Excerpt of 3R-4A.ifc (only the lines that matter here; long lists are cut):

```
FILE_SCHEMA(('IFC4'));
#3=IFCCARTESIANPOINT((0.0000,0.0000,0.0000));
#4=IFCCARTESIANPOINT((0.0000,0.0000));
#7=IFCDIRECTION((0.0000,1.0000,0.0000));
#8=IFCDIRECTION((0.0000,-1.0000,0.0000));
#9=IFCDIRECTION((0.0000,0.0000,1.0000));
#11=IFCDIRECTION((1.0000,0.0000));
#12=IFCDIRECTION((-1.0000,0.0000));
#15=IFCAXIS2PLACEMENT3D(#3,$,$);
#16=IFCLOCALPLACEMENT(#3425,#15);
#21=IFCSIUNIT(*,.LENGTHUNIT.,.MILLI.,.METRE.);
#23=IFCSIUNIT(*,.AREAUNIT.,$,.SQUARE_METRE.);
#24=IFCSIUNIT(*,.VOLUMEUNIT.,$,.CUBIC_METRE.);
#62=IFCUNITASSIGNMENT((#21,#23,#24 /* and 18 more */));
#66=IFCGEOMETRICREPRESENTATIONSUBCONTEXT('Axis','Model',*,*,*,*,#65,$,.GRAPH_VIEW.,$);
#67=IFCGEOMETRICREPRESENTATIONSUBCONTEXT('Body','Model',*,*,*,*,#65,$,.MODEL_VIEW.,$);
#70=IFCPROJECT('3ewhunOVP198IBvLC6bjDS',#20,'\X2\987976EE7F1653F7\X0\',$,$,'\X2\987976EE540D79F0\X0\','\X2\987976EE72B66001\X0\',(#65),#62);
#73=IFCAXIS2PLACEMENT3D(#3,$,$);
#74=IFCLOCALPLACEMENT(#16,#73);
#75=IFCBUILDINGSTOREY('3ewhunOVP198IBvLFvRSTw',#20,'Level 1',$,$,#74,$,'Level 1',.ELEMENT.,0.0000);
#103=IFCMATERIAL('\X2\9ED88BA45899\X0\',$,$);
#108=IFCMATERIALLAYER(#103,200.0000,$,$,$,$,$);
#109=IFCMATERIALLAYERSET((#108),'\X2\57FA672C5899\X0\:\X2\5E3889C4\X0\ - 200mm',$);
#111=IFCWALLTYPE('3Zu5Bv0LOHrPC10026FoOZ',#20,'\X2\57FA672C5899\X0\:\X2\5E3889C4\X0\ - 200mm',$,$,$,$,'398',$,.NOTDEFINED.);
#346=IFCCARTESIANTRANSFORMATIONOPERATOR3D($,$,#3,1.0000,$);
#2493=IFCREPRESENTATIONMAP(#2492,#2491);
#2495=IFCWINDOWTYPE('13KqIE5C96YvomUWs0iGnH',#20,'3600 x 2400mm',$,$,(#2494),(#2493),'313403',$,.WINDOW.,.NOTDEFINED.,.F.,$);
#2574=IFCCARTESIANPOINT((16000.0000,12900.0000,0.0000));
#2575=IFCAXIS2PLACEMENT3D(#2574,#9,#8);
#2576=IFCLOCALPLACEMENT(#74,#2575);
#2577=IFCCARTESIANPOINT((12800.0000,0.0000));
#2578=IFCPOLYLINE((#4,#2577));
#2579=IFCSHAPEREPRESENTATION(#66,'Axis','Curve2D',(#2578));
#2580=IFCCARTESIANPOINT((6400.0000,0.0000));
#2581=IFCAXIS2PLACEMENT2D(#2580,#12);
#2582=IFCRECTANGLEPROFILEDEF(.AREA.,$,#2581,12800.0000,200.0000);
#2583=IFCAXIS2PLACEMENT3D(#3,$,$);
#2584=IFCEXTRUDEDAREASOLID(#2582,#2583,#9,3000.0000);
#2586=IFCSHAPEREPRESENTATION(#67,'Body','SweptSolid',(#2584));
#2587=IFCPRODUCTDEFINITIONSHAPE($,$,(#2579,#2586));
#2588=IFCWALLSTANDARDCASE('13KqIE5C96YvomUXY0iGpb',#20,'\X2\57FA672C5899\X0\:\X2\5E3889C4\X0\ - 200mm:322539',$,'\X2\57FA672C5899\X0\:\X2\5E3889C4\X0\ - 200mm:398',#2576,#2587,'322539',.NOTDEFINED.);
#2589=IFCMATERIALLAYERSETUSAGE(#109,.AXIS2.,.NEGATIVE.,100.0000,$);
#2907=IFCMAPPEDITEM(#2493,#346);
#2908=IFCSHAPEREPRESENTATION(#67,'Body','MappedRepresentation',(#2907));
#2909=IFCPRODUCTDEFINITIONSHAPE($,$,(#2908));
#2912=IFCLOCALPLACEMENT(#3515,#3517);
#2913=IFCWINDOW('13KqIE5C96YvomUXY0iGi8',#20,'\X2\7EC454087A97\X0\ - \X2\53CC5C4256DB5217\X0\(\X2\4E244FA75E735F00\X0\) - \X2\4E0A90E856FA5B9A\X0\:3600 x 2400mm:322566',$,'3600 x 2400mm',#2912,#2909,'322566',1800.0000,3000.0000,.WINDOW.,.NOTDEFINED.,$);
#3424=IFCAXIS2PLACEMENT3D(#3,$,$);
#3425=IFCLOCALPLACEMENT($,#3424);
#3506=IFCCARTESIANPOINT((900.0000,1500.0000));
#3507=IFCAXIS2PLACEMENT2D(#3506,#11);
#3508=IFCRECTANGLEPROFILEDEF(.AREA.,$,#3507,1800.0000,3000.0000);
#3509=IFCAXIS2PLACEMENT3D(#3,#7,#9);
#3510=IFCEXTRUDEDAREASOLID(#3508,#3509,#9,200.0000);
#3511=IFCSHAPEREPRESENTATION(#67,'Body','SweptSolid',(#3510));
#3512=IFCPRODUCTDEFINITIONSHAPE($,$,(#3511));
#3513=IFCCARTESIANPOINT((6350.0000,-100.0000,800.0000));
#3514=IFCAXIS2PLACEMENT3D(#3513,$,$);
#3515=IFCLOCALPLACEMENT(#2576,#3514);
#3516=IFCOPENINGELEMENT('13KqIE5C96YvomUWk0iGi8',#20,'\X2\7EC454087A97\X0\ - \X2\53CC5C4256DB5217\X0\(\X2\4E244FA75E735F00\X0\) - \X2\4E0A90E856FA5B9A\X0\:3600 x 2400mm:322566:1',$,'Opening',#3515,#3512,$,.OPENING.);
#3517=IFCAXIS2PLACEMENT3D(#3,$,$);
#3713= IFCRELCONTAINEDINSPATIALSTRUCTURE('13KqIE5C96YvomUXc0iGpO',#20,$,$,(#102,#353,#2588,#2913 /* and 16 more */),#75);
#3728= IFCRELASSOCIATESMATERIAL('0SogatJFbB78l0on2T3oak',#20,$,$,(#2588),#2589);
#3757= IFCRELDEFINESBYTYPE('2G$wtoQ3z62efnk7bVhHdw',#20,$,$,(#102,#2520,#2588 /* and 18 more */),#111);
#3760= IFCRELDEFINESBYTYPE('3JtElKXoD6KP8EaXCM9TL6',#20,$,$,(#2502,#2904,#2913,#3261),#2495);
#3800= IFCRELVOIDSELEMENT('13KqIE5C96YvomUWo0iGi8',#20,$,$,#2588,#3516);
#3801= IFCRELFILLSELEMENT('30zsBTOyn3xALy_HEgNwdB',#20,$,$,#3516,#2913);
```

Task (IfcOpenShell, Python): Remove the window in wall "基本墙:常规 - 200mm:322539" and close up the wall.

```python
import ifcopenshell
import ifcopenshell.api.feature
import ifcopenshell.api.root
import ifcopenshell.geom
import ifcopenshell.util.shape

model = ifcopenshell.open("3R-4A.ifc")
settings = ifcopenshell.geom.settings()


def volume(element):
    """Net volume in cubic metres, openings subtracted."""
    shape = ifcopenshell.geom.create_shape(settings, element)
    return ifcopenshell.util.shape.get_volume(shape.geometry)


window = model.by_guid("13KqIE5C96YvomUXY0iGi8")
opening = window.FillsVoids[0].RelatingOpeningElement
wall = opening.VoidsElements[0].RelatingBuildingElement
before = volume(wall)

ifcopenshell.api.root.remove_product(model, product=window)
ifcopenshell.api.feature.remove_feature(model, feature=opening)

after = volume(wall)

print(f"wall volume {before:.3f} -> {after:.3f} m3")

model.write("3R-4A_updated.ifc")
```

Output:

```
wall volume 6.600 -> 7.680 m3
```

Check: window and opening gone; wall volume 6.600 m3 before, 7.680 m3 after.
